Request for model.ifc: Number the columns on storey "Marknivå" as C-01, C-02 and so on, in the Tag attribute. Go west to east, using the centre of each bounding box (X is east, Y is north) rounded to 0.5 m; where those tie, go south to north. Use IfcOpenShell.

First a look at what the model holds.

```python
import ifcopenshell
import ifcopenshell.util.element
import ifcopenshell.util.placement

model = ifcopenshell.open("model.ifc")
print(model.schema)
storey = next(s for s in model.by_type("IfcBuildingStorey") if s.Name == "Marknivå")
columns = [e for e in ifcopenshell.util.element.get_decomposition(storey) if e.is_a("IfcColumn")]
for e in sorted(columns, key=lambda e: e.id()):
    origin = ifcopenshell.util.placement.get_local_placement(e.ObjectPlacement)[:3, 3]
    print(e.id(), e.Tag, e.Name, origin.round(2) + 0.0, sep=" | ")
```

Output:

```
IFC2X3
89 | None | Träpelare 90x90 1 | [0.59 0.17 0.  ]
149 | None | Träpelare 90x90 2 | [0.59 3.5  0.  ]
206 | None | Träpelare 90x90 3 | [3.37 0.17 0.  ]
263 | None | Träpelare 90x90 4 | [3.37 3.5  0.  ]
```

```python
import ifcopenshell
import ifcopenshell.geom
import ifcopenshell.util.element
import ifcopenshell.util.shape

model = ifcopenshell.open("model.ifc")
settings = ifcopenshell.geom.settings()
settings.set("use-world-coords", True)


def centre(element):
    shape = ifcopenshell.geom.create_shape(settings, element)
    return ifcopenshell.util.shape.get_bbox_centroid(shape.geometry)


storey = next(s for s in model.by_type("IfcBuildingStorey") if s.Name == "Marknivå")
columns = [e for e in ifcopenshell.util.element.get_decomposition(storey) if e.is_a("IfcColumn")]

# Insertion points can sit at a corner or the storey origin, so sort by the geometry (in metres).
centres = {e: centre(e) for e in columns}
columns.sort(key=lambda e: (round(centres[e][0] / 0.5), centres[e][1]))

for i, e in enumerate(columns, start=1):
    number = f"C-{i:02d}"
    e.Tag = number
    print(e.id(), number)

model.write("model_rev.ifc")
```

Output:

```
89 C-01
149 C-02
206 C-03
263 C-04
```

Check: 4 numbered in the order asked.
